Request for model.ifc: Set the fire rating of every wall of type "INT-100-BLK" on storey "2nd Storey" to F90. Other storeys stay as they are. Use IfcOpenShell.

First a look at what the model holds.

```python
import ifcopenshell
import ifcopenshell.util.element

model = ifcopenshell.open("model.ifc")
print(model.schema)
storey = next(s for s in model.by_type("IfcBuildingStorey") if s.Name == "2nd Storey")
walls = [e for e in ifcopenshell.util.element.get_decomposition(storey) if e.is_a("IfcWall")]
seen = {}
for e in walls:
    element_type = ifcopenshell.util.element.get_type(e)
    key = (element_type.Name if element_type != e and element_type else None, ifcopenshell.util.element.get_pset(e, "Pset_WallCommon", "FireRating"))
    seen[key] = seen.get(key, 0) + 1
for (name, value), count in sorted(seen.items(), key=str):
    print(count, "x", name, "|", value)
```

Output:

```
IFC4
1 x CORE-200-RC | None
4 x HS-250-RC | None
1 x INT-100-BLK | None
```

```python
import ifcopenshell
import ifcopenshell.api.pset
import ifcopenshell.util.element

model = ifcopenshell.open("model.ifc")

storey = next(s for s in model.by_type("IfcBuildingStorey") if s.Name == "2nd Storey")
walls = [e for e in ifcopenshell.util.element.get_decomposition(storey) if e.is_a("IfcWall")]

count = 0
for e in walls:
    element_type = ifcopenshell.util.element.get_type(e)
    if element_type in (None, e) or element_type.Name != "INT-100-BLK":
        continue
    # add_pset returns the element's existing set when there is one.
    pset = ifcopenshell.api.pset.add_pset(model, product=e, name="Pset_WallCommon")
    ifcopenshell.api.pset.edit_pset(model, pset=pset, properties={"FireRating": "F90"})
    count += 1

print(count, "walls updated")

model.write("model_v2.ifc")
```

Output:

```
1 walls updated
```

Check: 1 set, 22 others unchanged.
